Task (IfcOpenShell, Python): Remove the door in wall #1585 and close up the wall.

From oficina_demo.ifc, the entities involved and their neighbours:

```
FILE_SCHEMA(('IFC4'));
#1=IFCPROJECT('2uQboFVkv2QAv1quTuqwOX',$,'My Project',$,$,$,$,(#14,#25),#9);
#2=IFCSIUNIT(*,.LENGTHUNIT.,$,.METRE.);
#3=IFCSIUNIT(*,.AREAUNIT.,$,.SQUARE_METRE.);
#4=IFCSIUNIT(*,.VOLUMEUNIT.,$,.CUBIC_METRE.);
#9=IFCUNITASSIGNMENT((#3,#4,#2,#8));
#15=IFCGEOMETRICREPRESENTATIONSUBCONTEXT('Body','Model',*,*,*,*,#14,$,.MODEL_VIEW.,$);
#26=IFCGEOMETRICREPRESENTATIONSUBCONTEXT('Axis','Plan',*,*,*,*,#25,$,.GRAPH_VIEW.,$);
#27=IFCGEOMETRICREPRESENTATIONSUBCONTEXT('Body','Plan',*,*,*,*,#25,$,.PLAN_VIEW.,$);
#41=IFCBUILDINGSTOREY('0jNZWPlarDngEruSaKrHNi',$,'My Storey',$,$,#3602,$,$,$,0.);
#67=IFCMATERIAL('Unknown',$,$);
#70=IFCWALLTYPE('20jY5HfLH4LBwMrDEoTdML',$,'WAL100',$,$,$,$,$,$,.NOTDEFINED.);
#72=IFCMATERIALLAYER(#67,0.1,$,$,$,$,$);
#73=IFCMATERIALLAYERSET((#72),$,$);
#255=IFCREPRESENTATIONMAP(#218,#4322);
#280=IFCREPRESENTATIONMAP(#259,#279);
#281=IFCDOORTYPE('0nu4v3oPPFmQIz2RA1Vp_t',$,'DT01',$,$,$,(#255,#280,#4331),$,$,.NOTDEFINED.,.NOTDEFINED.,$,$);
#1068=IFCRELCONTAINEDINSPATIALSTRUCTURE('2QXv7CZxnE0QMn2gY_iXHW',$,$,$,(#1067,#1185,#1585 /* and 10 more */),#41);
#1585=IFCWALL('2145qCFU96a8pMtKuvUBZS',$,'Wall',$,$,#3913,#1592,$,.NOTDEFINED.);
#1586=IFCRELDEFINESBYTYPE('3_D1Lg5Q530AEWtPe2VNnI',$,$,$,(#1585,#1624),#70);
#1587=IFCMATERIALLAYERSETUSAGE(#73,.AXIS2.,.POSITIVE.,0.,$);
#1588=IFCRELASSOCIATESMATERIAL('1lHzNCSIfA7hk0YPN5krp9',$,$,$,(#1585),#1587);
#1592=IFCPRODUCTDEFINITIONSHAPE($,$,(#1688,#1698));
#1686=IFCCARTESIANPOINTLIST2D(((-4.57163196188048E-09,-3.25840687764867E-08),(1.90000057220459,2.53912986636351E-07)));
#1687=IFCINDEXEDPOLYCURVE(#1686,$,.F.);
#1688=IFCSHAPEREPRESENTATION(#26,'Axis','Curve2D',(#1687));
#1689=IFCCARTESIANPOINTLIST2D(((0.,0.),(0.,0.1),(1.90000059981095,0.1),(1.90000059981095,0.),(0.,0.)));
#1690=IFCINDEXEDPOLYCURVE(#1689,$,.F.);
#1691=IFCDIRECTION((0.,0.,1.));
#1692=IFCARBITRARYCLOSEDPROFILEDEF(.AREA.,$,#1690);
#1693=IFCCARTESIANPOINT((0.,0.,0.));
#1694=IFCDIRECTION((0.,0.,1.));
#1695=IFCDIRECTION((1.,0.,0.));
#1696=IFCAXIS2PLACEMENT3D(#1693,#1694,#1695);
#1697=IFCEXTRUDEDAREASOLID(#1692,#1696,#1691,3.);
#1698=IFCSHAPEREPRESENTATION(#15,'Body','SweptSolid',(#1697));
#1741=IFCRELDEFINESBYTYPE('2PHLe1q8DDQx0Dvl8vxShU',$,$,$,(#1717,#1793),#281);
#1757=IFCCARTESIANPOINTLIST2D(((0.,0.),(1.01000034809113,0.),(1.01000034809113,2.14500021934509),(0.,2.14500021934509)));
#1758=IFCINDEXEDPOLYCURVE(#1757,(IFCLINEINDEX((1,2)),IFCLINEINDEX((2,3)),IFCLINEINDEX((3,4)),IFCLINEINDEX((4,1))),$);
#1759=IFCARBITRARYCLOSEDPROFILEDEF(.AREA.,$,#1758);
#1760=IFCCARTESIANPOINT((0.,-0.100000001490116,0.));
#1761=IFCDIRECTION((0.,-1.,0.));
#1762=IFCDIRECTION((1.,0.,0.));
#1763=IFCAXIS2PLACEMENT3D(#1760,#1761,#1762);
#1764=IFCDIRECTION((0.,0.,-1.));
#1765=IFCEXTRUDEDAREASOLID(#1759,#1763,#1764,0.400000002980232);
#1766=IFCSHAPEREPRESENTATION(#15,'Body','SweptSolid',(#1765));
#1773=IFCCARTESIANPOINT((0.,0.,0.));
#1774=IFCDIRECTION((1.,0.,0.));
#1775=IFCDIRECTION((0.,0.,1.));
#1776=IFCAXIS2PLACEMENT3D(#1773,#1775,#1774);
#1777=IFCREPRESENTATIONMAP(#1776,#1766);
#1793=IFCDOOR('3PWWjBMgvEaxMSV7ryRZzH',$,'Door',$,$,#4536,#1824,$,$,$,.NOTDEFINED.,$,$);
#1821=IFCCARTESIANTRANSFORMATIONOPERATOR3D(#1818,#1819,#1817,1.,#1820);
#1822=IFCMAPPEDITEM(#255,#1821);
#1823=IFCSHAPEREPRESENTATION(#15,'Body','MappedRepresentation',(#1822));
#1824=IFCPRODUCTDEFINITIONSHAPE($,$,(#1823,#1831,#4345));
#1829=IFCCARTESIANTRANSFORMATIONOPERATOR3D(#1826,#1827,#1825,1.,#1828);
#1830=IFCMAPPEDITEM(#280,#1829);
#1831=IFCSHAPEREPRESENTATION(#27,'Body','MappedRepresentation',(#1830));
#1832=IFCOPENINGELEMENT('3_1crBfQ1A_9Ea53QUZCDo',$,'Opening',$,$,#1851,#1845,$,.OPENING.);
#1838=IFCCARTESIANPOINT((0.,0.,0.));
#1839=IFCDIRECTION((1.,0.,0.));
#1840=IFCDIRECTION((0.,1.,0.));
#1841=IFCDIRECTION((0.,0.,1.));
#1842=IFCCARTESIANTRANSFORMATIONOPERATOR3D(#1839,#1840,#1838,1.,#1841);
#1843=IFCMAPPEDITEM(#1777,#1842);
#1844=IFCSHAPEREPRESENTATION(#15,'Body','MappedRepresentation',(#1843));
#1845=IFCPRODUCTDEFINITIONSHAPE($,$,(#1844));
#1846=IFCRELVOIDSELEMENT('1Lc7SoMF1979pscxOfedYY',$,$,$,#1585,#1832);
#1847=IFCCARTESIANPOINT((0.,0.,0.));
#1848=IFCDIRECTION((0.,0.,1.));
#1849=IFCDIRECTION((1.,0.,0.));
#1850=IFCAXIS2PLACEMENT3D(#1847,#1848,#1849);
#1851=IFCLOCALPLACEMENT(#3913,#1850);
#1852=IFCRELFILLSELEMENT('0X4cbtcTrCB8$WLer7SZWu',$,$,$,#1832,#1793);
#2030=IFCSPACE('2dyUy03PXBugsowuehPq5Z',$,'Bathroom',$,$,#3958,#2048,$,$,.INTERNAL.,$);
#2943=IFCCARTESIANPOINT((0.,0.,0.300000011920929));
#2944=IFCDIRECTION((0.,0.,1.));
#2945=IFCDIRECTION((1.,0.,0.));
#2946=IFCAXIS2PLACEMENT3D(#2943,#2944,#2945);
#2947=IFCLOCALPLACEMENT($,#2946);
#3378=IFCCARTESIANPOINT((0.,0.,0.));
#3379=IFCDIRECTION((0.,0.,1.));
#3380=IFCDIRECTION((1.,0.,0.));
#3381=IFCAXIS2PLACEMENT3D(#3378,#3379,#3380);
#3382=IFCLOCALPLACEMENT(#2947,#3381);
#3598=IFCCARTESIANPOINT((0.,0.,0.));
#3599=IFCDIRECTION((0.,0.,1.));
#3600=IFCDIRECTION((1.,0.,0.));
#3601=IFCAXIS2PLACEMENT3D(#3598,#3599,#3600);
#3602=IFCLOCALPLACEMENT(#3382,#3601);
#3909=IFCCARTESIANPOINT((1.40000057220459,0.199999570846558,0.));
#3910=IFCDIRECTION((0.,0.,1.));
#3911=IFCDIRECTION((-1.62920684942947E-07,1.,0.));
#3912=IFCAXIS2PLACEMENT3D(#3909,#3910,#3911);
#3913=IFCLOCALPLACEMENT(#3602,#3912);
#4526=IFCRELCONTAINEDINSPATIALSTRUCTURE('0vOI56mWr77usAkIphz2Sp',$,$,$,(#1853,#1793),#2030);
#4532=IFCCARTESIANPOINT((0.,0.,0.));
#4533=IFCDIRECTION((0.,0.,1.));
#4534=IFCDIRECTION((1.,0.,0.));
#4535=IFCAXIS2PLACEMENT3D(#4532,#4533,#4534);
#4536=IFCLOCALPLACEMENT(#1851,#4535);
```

```python
import ifcopenshell
import ifcopenshell.api.feature
import ifcopenshell.api.root
import ifcopenshell.geom
import ifcopenshell.util.shape

model = ifcopenshell.open("oficina_demo.ifc")
settings = ifcopenshell.geom.settings()


def volume(element):
    """Net volume in cubic metres, openings subtracted."""
    shape = ifcopenshell.geom.create_shape(settings, element)
    return ifcopenshell.util.shape.get_volume(shape.geometry)


door = model.by_guid("3PWWjBMgvEaxMSV7ryRZzH")
opening = door.FillsVoids[0].RelatingOpeningElement
wall = opening.VoidsElements[0].RelatingBuildingElement
before = volume(wall)

ifcopenshell.api.root.remove_product(model, product=door)
ifcopenshell.api.feature.remove_feature(model, feature=opening)

after = volume(wall)

print(f"wall volume {before:.3f} -> {after:.3f} m3")

model.write("oficina_demo_updated.ifc")
```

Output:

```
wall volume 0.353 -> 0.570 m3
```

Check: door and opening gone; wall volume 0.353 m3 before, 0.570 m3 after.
